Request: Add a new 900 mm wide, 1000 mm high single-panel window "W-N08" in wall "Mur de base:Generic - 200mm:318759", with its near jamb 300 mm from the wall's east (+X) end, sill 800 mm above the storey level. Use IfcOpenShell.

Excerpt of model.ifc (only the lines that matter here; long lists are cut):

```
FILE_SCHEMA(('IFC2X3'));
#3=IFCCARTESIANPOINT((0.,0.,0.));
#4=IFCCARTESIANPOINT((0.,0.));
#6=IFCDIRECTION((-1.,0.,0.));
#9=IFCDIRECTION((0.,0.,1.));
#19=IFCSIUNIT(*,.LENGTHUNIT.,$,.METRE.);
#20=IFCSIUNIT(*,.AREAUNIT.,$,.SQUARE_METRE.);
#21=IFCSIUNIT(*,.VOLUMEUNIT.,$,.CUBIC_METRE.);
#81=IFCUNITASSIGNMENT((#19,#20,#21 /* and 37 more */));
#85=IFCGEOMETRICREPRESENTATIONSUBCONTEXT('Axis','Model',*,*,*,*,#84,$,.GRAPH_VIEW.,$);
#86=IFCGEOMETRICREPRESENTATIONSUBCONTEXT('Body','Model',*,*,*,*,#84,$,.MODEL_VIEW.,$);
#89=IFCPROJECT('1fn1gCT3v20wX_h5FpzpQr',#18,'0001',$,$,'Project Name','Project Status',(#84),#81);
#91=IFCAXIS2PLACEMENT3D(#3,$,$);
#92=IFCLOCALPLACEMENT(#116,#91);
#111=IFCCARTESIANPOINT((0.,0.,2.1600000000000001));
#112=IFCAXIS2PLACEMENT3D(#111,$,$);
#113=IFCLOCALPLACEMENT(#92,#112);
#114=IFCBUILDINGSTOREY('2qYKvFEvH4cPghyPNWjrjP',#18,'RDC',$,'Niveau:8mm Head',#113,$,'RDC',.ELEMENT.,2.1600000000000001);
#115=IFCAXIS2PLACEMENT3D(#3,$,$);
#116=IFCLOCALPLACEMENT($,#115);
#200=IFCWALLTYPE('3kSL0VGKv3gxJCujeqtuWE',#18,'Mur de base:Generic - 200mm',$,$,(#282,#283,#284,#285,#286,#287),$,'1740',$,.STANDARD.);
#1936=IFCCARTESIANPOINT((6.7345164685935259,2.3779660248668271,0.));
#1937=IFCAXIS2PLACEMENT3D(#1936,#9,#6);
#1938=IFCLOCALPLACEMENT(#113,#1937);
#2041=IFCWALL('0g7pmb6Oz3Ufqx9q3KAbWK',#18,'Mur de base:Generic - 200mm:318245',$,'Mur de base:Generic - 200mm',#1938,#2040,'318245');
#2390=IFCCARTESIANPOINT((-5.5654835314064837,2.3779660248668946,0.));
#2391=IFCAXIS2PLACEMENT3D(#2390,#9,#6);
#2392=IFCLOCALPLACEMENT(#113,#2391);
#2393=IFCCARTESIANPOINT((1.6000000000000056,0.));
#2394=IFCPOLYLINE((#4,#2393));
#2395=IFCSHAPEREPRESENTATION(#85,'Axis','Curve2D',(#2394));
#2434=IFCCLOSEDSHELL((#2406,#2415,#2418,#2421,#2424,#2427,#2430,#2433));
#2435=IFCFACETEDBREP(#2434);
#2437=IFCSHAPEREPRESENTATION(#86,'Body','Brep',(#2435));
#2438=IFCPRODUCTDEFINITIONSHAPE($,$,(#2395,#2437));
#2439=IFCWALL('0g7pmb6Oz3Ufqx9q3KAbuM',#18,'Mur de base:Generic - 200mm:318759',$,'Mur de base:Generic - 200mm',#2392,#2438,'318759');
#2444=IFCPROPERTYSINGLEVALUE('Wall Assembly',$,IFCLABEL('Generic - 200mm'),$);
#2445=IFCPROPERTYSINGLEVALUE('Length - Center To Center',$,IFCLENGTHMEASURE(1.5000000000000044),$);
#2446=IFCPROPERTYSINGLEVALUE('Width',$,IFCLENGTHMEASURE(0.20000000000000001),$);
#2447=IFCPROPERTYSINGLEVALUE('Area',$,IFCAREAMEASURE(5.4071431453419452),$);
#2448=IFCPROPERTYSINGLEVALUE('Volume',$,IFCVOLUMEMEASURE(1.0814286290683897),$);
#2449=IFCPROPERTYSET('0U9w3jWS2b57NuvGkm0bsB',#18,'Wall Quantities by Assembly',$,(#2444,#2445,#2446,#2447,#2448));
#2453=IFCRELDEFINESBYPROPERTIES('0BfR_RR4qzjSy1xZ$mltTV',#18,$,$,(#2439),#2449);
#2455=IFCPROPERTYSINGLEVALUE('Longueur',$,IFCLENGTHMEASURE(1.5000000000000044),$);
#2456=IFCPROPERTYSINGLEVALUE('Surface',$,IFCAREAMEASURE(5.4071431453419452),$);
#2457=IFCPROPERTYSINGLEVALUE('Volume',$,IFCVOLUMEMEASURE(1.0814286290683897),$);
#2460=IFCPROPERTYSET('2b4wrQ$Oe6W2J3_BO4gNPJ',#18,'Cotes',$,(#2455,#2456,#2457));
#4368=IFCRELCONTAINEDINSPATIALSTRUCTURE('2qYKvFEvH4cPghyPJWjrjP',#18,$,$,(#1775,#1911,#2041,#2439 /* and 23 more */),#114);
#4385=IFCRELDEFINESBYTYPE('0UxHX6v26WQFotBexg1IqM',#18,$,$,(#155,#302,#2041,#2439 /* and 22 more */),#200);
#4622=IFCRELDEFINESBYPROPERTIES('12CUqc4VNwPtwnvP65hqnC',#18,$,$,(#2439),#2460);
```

```python
import numpy as np
import ifcopenshell
import ifcopenshell.api.feature
import ifcopenshell.api.geometry
import ifcopenshell.api.pset
import ifcopenshell.api.root
import ifcopenshell.api.spatial
import ifcopenshell.api.type
import ifcopenshell.geom
import ifcopenshell.util.element
import ifcopenshell.util.placement
import ifcopenshell.util.representation
import ifcopenshell.util.shape
import ifcopenshell.util.unit

model = ifcopenshell.open("model.ifc")
unit_scale = ifcopenshell.util.unit.calculate_unit_scale(model)
area_scale = ifcopenshell.util.unit.calculate_unit_scale(model, "AREAUNIT")
volume_scale = ifcopenshell.util.unit.calculate_unit_scale(model, "VOLUMEUNIT")
settings = ifcopenshell.geom.settings()


def volume(element):
    """Net volume in cubic metres, openings subtracted."""
    shape = ifcopenshell.geom.create_shape(settings, element)
    return ifcopenshell.util.shape.get_volume(shape.geometry)


wall = model.by_id(2439)
storey = ifcopenshell.util.element.get_container(wall, ifc_class="IfcBuildingStorey")
context = ifcopenshell.util.representation.get_context(model, "Model", "Body", "MODEL_VIEW")
before = volume(wall)

width, height, from_end, sill = 0.9, 1, 0.3, 0.8  # metres

# The wall runs along its own X axis, and the end named is its -X end.
wall_shape = ifcopenshell.geom.create_shape(settings, wall)
x, y, z = ifcopenshell.util.shape.get_vertices(wall_shape.geometry).T
start = x.min() + from_end
face, thickness = float(y.min()), float(y.max() - y.min())
wall_matrix = ifcopenshell.util.placement.get_local_placement(wall.ObjectPlacement)
level = ifcopenshell.util.placement.get_local_placement(storey.ObjectPlacement)[2, 3]


def in_wall(x, y):
    """Placement at x, y metres in the wall's axes, at sill height."""
    matrix = wall_matrix.copy()
    matrix[:, 3] = wall_matrix @ np.array([x / unit_scale, y / unit_scale, 0.0, 1.0])
    matrix[2, 3] = level + sill / unit_scale
    return matrix


# Opening: a box that overshoots both wall faces by 50 mm.
opening = ifcopenshell.api.root.create_entity(model, ifc_class="IfcOpeningElement")
box = ifcopenshell.api.geometry.add_wall_representation(
    model, context=context, length=width, height=height, thickness=thickness + 0.1
)
ifcopenshell.api.geometry.assign_representation(model, product=opening, representation=box)
ifcopenshell.api.geometry.edit_object_placement(model, product=opening, matrix=in_wall(start, face - 0.05), is_si=False)
ifcopenshell.api.feature.add_feature(model, feature=opening, element=wall)

window = ifcopenshell.api.root.create_entity(model, ifc_class="IfcWindow", name="W-N08")
window.OverallWidth, window.OverallHeight = width / unit_scale, height / unit_scale
body = ifcopenshell.api.geometry.add_window_representation(
    model,
    context=context,
    overall_width=window.OverallWidth,
    overall_height=window.OverallHeight,
    partition_type="SINGLE_PANEL",
)
ifcopenshell.api.geometry.assign_representation(model, product=window, representation=body)
ifcopenshell.api.spatial.assign_container(model, products=[window], relating_structure=storey)
fills = ifcopenshell.api.feature.add_filling(model, opening=opening, element=window)
fills.OwnerHistory = window.OwnerHistory  # required in IFC2X3

# IFC2X3 keeps the operation on the window style.
style = ifcopenshell.api.root.create_entity(model, ifc_class="IfcWindowStyle", name="W-N08")
style.OperationType, style.ConstructionType = "SINGLE_PANEL", "NOTDEFINED"
style.ParameterTakesPrecedence = style.Sizeable = False
ifcopenshell.api.type.assign_type(model, related_objects=[window], relating_type=style)

# Centre the window in the wall's thickness.
ifcopenshell.api.geometry.edit_object_placement(model, product=window, matrix=in_wall(start, face), is_si=False)
window_shape = ifcopenshell.geom.create_shape(settings, window)
depth = ifcopenshell.util.shape.get_vertices(window_shape.geometry)[:, 1]
offset = face + thickness / 2 - (depth.min() + depth.max()) / 2
ifcopenshell.api.geometry.edit_object_placement(model, product=window, matrix=in_wall(start, offset), is_si=False)

after = volume(wall)

# Update the wall's stored quantities.
pset = model.by_id(ifcopenshell.util.element.get_pset(wall, "Wall Quantities by Assembly", should_inherit=False)["id"])
ifcopenshell.api.pset.edit_pset(model, pset=pset, properties={
    "Area": model.create_entity("IfcAreaMeasure", after / thickness / area_scale),
    "Volume": model.create_entity("IfcVolumeMeasure", after / volume_scale),
})
pset = model.by_id(ifcopenshell.util.element.get_pset(wall, "Cotes", should_inherit=False)["id"])
ifcopenshell.api.pset.edit_pset(model, pset=pset, properties={
    "Surface": model.create_entity("IfcAreaMeasure", after / thickness / area_scale),
    "Volume": model.create_entity("IfcVolumeMeasure", after / volume_scale),
})

print(f"wall volume {before:.3f} -> {after:.3f} m3")

model.write("model_rev.ifc")
```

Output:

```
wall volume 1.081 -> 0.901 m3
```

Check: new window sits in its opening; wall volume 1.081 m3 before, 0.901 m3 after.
